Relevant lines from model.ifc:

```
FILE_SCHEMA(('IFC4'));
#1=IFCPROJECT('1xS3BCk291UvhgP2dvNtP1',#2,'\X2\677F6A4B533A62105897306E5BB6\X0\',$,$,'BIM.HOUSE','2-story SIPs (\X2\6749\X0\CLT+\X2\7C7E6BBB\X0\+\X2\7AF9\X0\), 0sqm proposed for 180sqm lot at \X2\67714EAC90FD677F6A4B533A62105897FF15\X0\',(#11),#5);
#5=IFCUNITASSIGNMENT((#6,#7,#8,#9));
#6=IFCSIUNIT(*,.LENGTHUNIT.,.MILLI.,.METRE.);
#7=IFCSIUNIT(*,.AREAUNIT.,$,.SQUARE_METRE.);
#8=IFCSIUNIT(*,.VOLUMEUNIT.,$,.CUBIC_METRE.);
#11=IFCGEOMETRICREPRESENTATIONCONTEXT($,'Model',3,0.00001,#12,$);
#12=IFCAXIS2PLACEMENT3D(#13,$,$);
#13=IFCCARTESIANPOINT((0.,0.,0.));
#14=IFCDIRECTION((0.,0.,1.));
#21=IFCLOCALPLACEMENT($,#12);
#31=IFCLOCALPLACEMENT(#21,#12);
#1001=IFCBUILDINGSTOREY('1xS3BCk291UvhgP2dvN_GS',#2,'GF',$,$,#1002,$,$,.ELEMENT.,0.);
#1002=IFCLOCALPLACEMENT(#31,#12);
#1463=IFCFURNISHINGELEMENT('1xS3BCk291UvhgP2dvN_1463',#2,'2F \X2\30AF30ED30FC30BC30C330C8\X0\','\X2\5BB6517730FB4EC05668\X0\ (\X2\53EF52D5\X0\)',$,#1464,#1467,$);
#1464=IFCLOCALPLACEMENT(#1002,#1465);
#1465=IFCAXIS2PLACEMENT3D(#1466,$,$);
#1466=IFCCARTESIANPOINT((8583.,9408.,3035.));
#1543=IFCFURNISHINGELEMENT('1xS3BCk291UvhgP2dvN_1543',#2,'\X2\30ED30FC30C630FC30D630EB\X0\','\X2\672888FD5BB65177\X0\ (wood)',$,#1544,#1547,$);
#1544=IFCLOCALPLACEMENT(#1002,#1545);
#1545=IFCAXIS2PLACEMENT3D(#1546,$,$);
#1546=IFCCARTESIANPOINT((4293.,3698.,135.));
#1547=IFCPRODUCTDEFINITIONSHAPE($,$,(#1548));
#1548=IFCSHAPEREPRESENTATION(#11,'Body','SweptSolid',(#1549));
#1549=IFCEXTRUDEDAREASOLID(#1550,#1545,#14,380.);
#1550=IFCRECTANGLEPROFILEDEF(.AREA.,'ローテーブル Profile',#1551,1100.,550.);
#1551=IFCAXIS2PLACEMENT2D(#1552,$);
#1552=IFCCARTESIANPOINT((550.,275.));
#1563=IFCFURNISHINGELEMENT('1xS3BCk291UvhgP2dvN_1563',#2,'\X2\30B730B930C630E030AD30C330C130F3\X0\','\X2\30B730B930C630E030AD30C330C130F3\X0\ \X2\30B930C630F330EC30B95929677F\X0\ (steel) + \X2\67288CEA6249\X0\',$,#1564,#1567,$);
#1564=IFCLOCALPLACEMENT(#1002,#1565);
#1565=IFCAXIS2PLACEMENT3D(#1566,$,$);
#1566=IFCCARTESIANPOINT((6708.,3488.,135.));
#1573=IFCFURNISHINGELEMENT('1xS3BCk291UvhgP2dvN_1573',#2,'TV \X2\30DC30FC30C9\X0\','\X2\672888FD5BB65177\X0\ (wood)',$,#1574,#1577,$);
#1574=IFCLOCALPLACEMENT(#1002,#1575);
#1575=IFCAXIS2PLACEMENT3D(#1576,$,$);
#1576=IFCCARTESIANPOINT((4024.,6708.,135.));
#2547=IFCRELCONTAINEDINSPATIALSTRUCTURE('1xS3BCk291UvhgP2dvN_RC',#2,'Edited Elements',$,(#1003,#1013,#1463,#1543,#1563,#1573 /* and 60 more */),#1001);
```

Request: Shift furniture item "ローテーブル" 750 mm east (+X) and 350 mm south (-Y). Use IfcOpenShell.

```python
import ifcopenshell
import ifcopenshell.api.geometry
import ifcopenshell.util.placement

model = ifcopenshell.open("model.ifc")

item = model.by_guid("1xS3BCk291UvhgP2dvN_1543")
matrix = ifcopenshell.util.placement.get_local_placement(item.ObjectPlacement)
matrix[0, 3] += 750.0
matrix[1, 3] -= 350.0
ifcopenshell.api.geometry.edit_object_placement(model, product=item, matrix=matrix, is_si=False)

print(ifcopenshell.util.placement.get_local_placement(item.ObjectPlacement).round(3) + 0.0)

model.write("model_v2.ifc")
```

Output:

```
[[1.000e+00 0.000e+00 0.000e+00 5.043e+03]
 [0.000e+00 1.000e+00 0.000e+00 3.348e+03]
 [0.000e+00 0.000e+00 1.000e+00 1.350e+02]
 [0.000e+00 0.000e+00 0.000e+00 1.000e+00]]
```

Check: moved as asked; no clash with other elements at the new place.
